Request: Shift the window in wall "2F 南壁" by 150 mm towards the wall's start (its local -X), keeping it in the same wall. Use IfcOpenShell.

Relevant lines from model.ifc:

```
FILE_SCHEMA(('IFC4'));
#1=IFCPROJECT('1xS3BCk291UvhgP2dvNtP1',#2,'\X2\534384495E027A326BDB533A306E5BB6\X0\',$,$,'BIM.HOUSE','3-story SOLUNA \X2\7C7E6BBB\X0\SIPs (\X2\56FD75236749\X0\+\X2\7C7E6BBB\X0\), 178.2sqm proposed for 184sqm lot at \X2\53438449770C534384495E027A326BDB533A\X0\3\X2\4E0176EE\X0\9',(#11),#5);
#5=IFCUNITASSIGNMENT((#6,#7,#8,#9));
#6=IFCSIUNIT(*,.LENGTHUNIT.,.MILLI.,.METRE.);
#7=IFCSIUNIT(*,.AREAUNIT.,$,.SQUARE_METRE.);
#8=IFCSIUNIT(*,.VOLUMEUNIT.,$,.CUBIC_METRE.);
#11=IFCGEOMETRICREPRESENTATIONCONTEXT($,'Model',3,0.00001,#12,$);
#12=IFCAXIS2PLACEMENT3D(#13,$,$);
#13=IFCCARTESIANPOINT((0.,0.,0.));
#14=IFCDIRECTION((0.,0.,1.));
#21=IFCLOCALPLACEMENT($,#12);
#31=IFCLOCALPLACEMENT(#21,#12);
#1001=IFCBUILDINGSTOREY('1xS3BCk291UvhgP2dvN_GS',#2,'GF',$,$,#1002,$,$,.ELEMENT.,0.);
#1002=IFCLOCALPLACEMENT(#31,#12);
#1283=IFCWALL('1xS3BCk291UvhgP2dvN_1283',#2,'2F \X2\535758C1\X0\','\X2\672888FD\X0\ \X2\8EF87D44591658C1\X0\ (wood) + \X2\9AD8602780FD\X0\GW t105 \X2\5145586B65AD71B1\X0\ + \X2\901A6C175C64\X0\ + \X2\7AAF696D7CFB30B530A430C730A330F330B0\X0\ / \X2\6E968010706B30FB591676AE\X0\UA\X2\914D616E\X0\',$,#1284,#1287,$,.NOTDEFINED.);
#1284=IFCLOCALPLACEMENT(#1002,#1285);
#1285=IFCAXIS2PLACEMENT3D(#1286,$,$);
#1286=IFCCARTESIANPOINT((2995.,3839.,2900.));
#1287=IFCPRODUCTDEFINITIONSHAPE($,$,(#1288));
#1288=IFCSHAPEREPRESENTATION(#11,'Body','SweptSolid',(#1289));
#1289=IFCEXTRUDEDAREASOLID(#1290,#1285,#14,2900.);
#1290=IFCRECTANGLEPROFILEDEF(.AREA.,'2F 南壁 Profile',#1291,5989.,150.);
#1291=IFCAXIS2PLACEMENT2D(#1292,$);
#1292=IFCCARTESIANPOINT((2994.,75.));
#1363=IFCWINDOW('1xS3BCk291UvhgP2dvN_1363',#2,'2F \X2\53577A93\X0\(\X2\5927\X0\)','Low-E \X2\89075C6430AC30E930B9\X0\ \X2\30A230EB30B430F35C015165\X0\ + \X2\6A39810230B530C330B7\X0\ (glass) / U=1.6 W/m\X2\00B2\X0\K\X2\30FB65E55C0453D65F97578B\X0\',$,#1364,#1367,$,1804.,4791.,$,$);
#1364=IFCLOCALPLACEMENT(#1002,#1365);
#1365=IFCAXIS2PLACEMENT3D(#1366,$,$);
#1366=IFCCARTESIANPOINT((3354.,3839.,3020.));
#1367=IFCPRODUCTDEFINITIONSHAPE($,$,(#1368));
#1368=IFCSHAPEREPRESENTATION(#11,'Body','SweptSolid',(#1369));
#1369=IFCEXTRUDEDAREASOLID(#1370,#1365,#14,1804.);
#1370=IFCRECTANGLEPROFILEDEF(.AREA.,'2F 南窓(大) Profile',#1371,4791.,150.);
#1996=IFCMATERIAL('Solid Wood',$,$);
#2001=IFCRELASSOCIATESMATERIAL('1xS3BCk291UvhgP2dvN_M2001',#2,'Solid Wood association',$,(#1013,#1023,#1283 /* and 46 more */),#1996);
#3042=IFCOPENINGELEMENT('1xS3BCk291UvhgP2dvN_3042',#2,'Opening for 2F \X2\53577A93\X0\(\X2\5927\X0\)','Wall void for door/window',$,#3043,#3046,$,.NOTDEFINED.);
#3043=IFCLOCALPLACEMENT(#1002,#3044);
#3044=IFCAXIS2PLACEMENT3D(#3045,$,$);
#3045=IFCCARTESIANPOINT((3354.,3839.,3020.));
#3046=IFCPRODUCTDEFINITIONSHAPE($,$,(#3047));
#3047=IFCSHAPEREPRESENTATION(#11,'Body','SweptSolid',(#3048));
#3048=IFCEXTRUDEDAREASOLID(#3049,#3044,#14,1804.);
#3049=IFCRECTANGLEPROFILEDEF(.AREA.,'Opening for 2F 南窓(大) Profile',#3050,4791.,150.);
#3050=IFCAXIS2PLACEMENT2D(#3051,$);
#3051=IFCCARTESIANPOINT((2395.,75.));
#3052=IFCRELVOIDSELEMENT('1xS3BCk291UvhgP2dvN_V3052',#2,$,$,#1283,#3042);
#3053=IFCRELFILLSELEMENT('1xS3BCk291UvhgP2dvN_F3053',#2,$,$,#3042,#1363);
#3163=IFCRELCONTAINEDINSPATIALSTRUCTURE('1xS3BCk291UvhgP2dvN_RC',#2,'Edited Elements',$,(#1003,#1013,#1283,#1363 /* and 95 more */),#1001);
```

```python
import ifcopenshell
import ifcopenshell.api.geometry
import ifcopenshell.util.placement
import ifcopenshell.util.unit

model = ifcopenshell.open("model.ifc")
unit_scale = ifcopenshell.util.unit.calculate_unit_scale(model)

window = model.by_guid("1xS3BCk291UvhgP2dvN_1363")
opening = window.FillsVoids[0].RelatingOpeningElement
wall = opening.VoidsElements[0].RelatingBuildingElement

wall_matrix = ifcopenshell.util.placement.get_local_placement(wall.ObjectPlacement)
shift = wall_matrix[:3, 0] * -0.15 / unit_scale
before = ifcopenshell.util.placement.get_local_placement(window.ObjectPlacement)[:3, 3].copy()

# The window is not placed relative to its opening, so move both.
for product in (opening, window):
    matrix = ifcopenshell.util.placement.get_local_placement(product.ObjectPlacement)
    matrix[:3, 3] += shift
    ifcopenshell.api.geometry.edit_object_placement(model, product=product, matrix=matrix, is_si=False)

after = ifcopenshell.util.placement.get_local_placement(window.ObjectPlacement)[:3, 3]
print("window moved by", (after - before).round(3) + 0.0)

model.write("model_edited.ifc")
```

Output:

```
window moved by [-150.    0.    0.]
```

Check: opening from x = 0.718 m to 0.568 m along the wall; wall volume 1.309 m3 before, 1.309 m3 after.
